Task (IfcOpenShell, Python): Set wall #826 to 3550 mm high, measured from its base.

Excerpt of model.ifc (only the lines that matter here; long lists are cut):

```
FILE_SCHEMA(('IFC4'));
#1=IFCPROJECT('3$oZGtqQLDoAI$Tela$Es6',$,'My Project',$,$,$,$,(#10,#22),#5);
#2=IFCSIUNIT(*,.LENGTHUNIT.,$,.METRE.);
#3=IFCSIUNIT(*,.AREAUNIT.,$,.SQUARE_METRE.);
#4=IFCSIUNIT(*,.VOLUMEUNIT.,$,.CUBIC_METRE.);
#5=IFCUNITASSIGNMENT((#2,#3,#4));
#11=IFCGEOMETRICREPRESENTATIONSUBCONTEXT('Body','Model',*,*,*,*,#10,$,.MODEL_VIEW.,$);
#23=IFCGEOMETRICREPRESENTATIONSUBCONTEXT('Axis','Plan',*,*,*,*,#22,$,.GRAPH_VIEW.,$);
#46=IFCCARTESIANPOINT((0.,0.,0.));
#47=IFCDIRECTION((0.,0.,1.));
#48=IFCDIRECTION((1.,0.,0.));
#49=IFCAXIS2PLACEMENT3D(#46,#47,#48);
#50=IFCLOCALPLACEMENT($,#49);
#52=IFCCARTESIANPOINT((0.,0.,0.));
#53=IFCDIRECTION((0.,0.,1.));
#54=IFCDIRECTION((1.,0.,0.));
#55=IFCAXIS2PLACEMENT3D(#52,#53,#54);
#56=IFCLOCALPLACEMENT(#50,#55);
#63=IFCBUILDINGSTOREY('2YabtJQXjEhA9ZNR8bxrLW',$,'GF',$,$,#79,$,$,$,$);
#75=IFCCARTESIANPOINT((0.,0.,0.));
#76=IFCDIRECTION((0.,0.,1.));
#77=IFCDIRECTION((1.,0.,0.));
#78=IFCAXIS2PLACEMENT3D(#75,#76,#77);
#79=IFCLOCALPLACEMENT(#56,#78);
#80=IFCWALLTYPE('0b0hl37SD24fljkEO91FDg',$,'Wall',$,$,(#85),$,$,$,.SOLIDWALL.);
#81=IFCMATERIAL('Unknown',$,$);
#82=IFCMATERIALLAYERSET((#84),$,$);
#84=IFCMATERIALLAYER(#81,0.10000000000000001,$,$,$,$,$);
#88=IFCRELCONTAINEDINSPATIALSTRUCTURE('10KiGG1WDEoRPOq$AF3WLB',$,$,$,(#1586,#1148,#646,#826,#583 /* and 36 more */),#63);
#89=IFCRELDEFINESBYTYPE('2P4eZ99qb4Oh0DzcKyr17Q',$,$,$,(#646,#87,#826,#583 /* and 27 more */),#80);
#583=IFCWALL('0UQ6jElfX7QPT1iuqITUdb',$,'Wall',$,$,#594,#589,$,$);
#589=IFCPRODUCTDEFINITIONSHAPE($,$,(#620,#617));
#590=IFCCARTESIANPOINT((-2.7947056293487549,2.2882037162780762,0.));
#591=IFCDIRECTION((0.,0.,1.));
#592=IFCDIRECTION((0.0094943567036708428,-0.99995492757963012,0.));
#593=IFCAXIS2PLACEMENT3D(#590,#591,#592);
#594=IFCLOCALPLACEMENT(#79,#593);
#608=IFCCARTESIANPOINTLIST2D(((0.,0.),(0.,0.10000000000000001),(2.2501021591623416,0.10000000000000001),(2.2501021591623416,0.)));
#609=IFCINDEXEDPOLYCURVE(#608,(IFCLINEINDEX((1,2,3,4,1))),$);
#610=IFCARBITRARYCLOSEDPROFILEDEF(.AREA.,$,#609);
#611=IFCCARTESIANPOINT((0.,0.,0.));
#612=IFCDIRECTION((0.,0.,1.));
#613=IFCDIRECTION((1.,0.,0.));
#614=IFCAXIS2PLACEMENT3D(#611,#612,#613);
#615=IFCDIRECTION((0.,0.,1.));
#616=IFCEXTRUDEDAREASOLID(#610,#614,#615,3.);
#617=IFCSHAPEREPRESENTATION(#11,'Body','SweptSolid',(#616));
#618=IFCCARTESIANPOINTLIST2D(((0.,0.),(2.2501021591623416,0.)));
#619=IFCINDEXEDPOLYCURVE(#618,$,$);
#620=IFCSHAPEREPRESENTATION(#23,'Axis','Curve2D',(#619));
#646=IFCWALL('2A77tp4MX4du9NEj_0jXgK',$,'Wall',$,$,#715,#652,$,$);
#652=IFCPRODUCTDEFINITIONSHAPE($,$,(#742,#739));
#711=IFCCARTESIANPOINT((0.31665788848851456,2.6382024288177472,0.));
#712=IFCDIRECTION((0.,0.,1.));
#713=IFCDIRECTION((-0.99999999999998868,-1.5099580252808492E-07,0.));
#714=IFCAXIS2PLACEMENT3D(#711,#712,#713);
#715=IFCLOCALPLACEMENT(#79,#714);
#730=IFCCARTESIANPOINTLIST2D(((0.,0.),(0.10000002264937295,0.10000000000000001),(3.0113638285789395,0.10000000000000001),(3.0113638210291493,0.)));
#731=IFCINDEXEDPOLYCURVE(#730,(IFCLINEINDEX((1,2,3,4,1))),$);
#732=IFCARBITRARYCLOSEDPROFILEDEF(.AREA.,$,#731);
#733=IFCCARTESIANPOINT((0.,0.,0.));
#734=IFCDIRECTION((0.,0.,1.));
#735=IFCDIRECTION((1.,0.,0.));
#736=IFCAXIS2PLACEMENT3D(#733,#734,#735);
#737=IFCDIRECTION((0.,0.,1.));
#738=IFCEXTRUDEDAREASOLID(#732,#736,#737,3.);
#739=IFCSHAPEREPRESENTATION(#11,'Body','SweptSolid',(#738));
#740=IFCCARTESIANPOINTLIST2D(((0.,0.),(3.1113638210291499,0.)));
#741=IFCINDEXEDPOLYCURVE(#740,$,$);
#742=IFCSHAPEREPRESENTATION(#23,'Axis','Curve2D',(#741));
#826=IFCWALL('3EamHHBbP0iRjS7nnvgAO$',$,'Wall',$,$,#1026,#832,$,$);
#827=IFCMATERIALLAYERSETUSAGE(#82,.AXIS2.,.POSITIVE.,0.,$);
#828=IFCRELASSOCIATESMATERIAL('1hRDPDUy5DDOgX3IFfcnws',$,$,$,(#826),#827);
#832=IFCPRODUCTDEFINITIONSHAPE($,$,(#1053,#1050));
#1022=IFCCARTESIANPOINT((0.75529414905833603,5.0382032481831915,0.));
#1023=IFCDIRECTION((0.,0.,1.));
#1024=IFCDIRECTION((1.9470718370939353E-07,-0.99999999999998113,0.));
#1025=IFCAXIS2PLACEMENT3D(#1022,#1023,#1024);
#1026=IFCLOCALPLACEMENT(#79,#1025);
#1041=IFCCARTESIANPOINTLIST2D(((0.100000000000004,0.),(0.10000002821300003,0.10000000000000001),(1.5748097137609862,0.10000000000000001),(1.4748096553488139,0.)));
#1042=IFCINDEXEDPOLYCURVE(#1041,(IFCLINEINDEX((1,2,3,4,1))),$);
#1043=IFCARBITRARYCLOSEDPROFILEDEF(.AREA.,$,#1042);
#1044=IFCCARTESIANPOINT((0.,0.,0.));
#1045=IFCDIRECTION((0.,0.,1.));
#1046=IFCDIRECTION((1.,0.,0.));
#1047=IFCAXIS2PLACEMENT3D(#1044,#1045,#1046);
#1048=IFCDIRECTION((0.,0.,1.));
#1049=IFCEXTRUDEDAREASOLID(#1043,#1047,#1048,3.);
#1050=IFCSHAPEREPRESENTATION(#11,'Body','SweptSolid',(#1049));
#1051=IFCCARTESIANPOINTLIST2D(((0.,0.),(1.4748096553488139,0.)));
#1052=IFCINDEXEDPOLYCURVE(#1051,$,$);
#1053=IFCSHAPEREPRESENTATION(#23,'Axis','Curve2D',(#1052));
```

```python
import ifcopenshell
import ifcopenshell.geom
import ifcopenshell.util.representation
import ifcopenshell.util.shape
import ifcopenshell.util.unit

model = ifcopenshell.open("model.ifc")
unit_scale = ifcopenshell.util.unit.calculate_unit_scale(model)
settings = ifcopenshell.geom.settings()


def volume(element):
    """Net volume in cubic metres, openings subtracted."""
    shape = ifcopenshell.geom.create_shape(settings, element)
    return ifcopenshell.util.shape.get_volume(shape.geometry)


wall = model.by_guid("3EamHHBbP0iRjS7nnvgAO$")
before = volume(wall)

body = ifcopenshell.util.representation.get_representation(wall, "Model", "Body")
solid = body.Items[0]
old_height = solid.Depth
solid.Depth = 3.55 / unit_scale
after = volume(wall)

print(f"height {old_height:g} -> {solid.Depth:g}, volume {before:.3f} -> {after:.3f} m3")

model.write("model-out.ifc")
```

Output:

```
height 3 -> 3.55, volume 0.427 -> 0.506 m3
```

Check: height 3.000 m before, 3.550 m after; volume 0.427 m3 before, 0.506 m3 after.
